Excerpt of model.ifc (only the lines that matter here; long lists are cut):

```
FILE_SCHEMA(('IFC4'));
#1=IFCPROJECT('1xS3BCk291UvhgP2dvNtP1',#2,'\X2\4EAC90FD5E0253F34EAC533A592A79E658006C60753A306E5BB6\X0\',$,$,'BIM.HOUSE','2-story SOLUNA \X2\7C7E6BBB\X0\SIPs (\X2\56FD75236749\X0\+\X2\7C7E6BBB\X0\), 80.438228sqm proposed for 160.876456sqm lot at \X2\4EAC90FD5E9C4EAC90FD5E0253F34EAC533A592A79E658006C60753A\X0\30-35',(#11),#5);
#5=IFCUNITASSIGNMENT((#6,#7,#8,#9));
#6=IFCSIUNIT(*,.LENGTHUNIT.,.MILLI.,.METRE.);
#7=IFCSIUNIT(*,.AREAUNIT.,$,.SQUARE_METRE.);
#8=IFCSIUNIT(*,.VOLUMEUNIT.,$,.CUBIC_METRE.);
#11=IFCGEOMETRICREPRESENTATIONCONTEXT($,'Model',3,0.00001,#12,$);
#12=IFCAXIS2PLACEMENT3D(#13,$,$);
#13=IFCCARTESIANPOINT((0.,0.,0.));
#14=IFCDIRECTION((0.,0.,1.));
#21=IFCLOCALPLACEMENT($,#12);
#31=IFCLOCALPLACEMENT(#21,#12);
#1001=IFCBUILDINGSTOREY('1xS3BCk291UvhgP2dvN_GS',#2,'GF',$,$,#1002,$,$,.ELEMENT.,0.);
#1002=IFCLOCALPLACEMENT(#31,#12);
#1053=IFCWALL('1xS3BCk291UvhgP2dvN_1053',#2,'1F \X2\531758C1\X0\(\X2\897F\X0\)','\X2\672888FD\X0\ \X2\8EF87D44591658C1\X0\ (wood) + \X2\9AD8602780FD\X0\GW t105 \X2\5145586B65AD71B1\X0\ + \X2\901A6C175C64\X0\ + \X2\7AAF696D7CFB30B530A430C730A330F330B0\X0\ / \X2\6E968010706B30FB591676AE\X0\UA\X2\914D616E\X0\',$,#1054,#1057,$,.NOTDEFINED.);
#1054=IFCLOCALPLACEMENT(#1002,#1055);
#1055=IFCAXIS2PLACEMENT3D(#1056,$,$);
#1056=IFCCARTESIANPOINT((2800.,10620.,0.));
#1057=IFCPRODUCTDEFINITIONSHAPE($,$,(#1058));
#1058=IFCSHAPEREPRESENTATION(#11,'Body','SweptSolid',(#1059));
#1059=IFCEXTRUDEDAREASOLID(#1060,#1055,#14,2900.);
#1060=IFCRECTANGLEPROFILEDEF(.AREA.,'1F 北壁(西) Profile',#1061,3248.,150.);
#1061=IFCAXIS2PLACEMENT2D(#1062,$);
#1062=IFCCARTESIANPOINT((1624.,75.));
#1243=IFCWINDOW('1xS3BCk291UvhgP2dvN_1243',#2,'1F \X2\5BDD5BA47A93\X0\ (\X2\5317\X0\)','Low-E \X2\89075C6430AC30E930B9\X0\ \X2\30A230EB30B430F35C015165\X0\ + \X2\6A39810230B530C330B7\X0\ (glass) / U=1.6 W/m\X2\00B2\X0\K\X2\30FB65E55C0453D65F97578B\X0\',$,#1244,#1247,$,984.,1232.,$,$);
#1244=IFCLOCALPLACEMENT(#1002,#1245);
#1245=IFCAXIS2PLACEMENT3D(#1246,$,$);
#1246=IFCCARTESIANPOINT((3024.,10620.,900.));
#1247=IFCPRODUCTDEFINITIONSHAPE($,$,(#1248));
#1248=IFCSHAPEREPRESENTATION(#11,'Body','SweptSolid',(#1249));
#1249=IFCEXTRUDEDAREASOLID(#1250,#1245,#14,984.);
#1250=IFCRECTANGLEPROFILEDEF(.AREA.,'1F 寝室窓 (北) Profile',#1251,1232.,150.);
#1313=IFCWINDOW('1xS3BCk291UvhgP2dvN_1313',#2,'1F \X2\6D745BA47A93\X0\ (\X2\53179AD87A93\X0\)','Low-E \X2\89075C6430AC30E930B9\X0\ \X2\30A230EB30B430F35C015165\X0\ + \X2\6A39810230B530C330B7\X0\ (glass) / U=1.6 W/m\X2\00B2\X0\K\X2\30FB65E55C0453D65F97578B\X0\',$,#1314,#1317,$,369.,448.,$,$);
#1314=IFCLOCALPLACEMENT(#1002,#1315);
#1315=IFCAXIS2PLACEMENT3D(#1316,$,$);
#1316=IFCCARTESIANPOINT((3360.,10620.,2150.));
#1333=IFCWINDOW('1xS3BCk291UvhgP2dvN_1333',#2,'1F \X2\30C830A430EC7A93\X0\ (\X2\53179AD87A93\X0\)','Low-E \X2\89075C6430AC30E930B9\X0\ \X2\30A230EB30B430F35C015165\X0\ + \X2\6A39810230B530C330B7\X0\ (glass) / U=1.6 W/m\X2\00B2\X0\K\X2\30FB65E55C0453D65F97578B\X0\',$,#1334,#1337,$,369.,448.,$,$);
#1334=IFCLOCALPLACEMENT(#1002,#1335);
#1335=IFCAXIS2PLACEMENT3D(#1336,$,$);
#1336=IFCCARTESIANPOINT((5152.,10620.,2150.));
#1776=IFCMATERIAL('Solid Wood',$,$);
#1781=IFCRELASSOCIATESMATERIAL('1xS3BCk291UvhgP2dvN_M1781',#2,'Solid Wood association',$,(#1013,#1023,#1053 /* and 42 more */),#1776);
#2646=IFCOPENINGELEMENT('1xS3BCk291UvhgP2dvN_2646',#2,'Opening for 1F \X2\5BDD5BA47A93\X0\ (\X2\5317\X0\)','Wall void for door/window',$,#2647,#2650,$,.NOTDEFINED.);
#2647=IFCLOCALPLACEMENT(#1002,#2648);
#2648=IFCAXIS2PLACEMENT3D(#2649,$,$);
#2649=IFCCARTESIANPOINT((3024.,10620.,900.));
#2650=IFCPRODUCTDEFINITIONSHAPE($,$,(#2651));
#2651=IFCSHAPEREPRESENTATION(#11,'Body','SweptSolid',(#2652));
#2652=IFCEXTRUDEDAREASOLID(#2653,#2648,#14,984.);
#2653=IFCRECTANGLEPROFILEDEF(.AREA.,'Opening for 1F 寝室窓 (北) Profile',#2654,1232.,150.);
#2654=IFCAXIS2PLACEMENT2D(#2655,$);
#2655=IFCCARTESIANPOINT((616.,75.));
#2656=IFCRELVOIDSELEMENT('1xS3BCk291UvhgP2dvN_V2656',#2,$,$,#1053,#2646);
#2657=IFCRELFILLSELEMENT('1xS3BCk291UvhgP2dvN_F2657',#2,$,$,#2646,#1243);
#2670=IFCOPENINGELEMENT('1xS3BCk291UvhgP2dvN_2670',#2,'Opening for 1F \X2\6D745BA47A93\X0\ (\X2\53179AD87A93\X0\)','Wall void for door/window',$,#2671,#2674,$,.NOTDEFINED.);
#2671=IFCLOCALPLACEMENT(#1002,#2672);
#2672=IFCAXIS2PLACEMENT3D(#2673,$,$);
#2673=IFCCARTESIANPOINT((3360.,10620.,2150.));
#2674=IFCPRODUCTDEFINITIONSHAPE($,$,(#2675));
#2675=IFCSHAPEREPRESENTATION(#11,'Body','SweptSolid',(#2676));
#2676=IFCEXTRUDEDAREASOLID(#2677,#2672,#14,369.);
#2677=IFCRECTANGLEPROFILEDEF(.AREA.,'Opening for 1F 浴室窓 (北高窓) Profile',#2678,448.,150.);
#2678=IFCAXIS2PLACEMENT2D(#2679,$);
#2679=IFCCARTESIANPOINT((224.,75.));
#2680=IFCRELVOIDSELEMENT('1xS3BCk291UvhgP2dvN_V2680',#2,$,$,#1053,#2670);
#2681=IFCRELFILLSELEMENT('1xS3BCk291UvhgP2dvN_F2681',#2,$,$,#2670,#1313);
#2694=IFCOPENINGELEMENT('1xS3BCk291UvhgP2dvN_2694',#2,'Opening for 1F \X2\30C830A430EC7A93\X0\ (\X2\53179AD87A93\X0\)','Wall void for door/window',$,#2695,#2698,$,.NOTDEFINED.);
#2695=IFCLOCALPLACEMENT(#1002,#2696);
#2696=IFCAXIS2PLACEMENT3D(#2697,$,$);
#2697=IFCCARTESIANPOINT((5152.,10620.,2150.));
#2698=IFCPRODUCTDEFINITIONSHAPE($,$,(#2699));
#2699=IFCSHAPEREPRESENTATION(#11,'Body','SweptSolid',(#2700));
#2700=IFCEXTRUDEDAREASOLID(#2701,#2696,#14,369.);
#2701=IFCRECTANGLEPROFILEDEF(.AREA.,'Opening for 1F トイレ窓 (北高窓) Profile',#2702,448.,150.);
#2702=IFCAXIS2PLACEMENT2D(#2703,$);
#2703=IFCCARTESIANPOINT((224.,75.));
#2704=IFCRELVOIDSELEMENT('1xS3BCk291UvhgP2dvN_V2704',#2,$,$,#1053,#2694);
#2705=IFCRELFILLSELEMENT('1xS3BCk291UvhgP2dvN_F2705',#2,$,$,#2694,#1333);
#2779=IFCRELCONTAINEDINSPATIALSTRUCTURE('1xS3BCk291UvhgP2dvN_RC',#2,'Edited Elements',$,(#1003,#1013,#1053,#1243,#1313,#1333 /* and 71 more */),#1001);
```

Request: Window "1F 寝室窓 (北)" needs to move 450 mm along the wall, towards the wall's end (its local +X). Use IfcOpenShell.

```python
import ifcopenshell
import ifcopenshell.api.geometry
import ifcopenshell.util.placement

model = ifcopenshell.open("model.ifc")

window = model.by_guid("1xS3BCk291UvhgP2dvN_1243")
opening = window.FillsVoids[0].RelatingOpeningElement
wall = opening.VoidsElements[0].RelatingBuildingElement

wall_matrix = ifcopenshell.util.placement.get_local_placement(wall.ObjectPlacement)
shift = wall_matrix[:3, 0] * 450.0
before = ifcopenshell.util.placement.get_local_placement(window.ObjectPlacement)[:3, 3].copy()

# The window is not placed relative to its opening, so move both.
for product in (opening, window):
    matrix = ifcopenshell.util.placement.get_local_placement(product.ObjectPlacement)
    matrix[:3, 3] += shift
    ifcopenshell.api.geometry.edit_object_placement(model, product=product, matrix=matrix, is_si=False)

after = ifcopenshell.util.placement.get_local_placement(window.ObjectPlacement)[:3, 3]
print("window moved by", (after - before).round(3) + 0.0)

model.write("model-out.ifc")
```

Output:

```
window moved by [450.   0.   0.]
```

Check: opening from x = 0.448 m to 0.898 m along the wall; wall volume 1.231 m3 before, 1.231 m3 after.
